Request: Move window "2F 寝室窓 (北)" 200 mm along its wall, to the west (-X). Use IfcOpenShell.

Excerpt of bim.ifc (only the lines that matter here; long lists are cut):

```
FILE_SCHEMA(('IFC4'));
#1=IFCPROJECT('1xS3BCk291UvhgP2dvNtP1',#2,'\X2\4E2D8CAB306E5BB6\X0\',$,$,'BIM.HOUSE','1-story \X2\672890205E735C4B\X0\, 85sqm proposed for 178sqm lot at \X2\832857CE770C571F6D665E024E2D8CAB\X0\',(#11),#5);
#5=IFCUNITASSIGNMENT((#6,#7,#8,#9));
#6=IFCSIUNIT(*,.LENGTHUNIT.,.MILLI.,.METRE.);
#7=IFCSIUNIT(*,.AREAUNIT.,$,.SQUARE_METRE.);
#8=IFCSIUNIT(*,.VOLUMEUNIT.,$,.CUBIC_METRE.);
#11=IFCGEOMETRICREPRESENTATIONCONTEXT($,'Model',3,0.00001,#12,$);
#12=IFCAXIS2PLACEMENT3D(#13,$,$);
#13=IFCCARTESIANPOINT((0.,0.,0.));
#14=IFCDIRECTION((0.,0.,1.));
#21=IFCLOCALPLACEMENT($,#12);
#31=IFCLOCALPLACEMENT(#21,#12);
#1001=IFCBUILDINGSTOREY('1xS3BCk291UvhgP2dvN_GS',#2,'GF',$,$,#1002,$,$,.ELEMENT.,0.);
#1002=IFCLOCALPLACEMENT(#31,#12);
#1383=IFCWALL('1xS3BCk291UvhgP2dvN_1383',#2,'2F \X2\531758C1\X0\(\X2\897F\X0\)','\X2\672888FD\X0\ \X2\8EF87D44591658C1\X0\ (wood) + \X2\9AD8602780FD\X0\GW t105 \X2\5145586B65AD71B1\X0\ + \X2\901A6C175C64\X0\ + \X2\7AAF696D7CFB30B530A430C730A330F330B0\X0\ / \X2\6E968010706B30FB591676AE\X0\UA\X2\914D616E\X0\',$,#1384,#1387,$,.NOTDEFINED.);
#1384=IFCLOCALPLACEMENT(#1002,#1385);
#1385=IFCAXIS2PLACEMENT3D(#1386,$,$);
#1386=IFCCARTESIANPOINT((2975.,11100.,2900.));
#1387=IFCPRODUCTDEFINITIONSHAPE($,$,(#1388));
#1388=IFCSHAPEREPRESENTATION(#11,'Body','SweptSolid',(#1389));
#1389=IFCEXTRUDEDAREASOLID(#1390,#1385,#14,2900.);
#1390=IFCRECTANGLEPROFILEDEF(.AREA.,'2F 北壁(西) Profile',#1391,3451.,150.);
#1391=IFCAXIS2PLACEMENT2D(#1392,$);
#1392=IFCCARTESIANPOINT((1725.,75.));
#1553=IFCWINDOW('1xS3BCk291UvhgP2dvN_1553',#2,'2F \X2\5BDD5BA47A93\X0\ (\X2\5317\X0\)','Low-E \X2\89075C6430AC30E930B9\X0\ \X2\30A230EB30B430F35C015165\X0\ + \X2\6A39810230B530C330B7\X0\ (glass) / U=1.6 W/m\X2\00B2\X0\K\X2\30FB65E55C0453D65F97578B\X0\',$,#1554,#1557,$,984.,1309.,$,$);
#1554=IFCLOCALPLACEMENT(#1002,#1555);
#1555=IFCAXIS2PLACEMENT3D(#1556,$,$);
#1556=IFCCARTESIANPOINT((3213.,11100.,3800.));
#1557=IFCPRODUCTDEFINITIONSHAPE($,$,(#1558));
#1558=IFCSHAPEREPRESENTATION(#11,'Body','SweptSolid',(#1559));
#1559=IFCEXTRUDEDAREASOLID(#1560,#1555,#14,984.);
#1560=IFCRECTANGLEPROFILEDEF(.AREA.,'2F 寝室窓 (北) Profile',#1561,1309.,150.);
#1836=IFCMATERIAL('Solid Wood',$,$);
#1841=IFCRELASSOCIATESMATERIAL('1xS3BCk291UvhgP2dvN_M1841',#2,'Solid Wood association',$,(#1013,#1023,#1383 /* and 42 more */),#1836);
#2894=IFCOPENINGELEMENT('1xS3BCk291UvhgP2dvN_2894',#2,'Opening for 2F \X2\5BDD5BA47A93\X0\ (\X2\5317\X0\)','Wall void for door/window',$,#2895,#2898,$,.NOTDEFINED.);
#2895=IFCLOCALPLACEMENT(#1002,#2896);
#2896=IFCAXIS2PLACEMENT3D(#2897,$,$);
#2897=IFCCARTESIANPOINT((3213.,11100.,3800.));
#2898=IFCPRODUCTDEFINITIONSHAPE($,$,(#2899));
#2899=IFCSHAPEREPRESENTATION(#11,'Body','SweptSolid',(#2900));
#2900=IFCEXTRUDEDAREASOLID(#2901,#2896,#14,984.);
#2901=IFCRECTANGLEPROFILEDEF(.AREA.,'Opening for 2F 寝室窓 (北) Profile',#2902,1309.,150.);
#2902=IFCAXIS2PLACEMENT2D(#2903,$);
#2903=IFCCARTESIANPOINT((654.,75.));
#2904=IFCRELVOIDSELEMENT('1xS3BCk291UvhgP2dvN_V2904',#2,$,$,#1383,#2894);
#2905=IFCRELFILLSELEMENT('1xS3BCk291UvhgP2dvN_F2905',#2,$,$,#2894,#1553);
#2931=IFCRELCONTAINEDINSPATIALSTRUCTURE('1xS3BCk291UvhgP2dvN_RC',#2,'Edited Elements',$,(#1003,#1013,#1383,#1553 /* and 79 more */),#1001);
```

```python
import ifcopenshell
import ifcopenshell.api.geometry
import ifcopenshell.util.placement

model = ifcopenshell.open("bim.ifc")

window = model.by_guid("1xS3BCk291UvhgP2dvN_1553")
opening = window.FillsVoids[0].RelatingOpeningElement
wall = opening.VoidsElements[0].RelatingBuildingElement

wall_matrix = ifcopenshell.util.placement.get_local_placement(wall.ObjectPlacement)
shift = wall_matrix[:3, 0] * -200.0
before = ifcopenshell.util.placement.get_local_placement(window.ObjectPlacement)[:3, 3].copy()

# The window is not placed relative to its opening, so move both.
for product in (opening, window):
    matrix = ifcopenshell.util.placement.get_local_placement(product.ObjectPlacement)
    matrix[:3, 3] += shift
    ifcopenshell.api.geometry.edit_object_placement(model, product=product, matrix=matrix, is_si=False)

after = ifcopenshell.util.placement.get_local_placement(window.ObjectPlacement)[:3, 3]
print("window moved by", (after - before).round(3) + 0.0)

model.write("bim_edited.ifc")
```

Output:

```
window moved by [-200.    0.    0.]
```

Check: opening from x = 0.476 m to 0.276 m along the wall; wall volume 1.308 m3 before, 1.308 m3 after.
